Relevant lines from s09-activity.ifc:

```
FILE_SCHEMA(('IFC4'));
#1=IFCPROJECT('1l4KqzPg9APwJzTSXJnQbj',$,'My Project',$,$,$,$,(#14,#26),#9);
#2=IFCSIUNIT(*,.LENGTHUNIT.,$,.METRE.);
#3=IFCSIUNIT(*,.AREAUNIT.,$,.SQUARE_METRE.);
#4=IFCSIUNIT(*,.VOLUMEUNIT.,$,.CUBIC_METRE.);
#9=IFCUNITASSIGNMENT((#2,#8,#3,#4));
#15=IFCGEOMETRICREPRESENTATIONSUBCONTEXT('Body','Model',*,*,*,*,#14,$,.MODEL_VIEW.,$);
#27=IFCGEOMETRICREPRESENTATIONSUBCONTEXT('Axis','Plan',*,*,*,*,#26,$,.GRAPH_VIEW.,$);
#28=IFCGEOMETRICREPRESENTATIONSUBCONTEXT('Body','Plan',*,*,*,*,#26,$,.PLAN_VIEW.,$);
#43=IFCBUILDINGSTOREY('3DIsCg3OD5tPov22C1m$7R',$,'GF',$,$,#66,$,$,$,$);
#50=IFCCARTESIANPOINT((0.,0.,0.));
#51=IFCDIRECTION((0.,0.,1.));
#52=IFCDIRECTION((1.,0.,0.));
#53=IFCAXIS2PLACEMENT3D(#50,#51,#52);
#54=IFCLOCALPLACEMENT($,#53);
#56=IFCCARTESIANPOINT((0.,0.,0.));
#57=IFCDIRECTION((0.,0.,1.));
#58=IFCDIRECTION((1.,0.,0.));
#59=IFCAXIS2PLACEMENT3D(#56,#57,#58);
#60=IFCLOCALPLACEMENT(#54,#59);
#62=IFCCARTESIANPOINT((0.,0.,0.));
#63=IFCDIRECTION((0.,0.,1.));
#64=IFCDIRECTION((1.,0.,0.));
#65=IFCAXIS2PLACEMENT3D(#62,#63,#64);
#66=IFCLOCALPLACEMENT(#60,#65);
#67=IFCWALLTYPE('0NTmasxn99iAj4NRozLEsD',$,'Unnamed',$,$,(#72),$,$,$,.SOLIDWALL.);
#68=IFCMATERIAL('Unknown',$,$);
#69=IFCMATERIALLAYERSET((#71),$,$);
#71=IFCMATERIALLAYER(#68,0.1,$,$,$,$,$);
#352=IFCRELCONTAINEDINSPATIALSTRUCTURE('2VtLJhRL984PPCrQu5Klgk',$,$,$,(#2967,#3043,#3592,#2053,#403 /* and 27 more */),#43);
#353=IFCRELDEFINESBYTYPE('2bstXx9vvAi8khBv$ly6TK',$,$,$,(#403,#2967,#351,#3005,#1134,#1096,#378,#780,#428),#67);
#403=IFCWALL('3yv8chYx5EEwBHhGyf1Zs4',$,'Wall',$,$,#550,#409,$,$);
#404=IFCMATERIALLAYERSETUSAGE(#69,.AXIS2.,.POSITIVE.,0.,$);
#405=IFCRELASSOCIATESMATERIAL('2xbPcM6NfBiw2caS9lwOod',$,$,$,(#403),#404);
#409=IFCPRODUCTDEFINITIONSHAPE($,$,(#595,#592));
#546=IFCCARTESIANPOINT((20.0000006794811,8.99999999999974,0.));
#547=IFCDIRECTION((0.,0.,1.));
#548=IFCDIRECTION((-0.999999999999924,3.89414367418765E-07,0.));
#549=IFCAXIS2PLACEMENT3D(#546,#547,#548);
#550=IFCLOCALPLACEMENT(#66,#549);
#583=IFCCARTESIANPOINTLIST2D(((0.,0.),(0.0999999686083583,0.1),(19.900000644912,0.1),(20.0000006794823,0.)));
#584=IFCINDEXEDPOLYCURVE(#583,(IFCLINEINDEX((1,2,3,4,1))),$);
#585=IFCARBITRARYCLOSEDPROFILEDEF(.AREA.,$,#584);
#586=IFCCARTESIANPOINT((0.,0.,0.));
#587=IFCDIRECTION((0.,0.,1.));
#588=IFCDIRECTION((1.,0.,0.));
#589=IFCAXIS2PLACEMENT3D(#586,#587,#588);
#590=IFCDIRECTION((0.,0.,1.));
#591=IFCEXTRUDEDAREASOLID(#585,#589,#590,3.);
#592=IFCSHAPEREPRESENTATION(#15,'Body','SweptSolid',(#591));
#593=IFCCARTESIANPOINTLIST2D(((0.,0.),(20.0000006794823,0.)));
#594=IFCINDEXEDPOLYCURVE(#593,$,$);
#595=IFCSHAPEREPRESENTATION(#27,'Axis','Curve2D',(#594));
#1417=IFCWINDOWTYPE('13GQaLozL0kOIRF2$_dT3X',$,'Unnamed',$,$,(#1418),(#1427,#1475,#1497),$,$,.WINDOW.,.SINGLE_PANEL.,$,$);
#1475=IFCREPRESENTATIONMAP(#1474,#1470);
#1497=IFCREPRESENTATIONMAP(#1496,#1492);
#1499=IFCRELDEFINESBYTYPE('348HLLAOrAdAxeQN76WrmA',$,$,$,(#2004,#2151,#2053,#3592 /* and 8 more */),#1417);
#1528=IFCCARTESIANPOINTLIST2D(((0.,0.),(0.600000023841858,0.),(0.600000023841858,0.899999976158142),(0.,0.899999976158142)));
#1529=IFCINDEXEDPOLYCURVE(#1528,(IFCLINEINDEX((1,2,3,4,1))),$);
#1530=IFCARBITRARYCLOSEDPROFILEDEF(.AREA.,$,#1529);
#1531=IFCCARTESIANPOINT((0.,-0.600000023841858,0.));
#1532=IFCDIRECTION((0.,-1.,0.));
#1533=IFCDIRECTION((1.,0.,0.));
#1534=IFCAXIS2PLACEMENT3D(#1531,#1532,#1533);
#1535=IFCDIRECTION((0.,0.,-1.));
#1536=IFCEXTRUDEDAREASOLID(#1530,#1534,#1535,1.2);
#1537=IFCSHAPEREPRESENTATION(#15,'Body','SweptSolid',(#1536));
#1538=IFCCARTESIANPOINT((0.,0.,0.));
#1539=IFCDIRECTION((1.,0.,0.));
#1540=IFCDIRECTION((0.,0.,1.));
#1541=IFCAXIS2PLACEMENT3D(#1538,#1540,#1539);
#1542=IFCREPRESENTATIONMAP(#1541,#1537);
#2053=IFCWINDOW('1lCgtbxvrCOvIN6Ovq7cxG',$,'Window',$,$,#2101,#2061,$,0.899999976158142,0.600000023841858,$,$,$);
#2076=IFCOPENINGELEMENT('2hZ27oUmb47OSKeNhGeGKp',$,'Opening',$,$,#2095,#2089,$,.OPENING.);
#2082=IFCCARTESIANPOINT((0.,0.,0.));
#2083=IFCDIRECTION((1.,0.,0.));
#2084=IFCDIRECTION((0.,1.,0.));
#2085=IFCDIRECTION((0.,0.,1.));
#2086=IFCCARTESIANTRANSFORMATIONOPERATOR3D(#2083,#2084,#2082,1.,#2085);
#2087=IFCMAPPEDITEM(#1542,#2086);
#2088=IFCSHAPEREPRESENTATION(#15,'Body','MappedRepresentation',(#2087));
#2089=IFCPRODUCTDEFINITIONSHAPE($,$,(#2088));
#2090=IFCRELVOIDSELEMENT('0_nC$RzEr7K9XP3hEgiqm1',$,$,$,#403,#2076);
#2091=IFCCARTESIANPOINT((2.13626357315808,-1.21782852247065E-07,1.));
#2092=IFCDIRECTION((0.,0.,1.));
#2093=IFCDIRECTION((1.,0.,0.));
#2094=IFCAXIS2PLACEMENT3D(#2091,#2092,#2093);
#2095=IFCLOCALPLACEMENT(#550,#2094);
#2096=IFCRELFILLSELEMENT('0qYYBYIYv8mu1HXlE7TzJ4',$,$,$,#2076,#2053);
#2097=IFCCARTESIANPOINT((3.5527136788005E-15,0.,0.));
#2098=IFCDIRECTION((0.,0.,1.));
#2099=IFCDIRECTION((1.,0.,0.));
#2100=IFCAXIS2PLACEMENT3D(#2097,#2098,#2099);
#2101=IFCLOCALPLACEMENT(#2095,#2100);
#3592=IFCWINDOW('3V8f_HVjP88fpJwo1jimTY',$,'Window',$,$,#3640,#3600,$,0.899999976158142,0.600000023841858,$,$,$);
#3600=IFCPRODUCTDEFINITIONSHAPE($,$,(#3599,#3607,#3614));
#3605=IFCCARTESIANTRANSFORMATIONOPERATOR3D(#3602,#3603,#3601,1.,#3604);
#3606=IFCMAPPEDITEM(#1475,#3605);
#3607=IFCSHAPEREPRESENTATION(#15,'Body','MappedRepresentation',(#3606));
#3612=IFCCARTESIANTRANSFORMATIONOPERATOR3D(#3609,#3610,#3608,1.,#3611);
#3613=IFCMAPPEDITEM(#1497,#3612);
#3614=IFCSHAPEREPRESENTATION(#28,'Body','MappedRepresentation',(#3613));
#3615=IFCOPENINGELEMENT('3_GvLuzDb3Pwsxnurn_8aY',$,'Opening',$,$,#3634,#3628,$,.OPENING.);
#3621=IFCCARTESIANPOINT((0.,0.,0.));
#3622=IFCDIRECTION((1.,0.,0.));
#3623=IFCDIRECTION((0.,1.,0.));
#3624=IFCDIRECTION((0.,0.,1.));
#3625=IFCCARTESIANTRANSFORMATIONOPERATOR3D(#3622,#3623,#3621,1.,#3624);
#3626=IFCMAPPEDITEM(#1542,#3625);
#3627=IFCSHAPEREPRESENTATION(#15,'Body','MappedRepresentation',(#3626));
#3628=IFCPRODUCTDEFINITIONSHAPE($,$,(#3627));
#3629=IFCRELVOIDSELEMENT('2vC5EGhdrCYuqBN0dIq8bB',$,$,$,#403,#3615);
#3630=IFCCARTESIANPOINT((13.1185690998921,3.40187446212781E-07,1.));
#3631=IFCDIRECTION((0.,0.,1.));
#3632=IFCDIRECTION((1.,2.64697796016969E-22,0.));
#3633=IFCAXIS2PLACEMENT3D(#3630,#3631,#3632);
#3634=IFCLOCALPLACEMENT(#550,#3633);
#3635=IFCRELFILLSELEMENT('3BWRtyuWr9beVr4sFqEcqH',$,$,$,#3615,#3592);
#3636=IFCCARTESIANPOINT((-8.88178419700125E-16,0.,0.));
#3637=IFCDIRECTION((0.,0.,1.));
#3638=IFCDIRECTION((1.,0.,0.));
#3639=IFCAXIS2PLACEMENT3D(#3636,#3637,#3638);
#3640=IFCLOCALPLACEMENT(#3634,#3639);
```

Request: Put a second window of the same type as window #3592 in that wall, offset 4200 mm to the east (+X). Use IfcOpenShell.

```python
import ifcopenshell
import ifcopenshell.api.feature
import ifcopenshell.api.geometry
import ifcopenshell.api.root
import ifcopenshell.geom
import ifcopenshell.util.element
import ifcopenshell.util.placement
import ifcopenshell.util.shape

model = ifcopenshell.open("s09-activity.ifc")
settings = ifcopenshell.geom.settings()


def volume(element):
    """Net volume in cubic metres, openings subtracted."""
    shape = ifcopenshell.geom.create_shape(settings, element)
    return ifcopenshell.util.shape.get_volume(shape.geometry)


window = model.by_guid("3V8f_HVjP88fpJwo1jimTY")
opening = window.FillsVoids[0].RelatingOpeningElement
wall = opening.VoidsElements[0].RelatingBuildingElement
before = volume(wall)
shift = ifcopenshell.util.placement.get_local_placement(wall.ObjectPlacement)[:3, 0] * -4.2

# copy_class copies the void relationship, type, container and properties, but no geometry.
new_opening = ifcopenshell.api.root.copy_class(model, product=opening)
new_opening.Representation = ifcopenshell.util.element.copy_deep(
    model, opening.Representation, exclude=["IfcGeometricRepresentationContext", "IfcRepresentationMap"]
)
new_window = ifcopenshell.api.root.copy_class(model, product=window)
new_window.Representation = ifcopenshell.util.element.copy_deep(
    model, window.Representation, exclude=["IfcGeometricRepresentationContext", "IfcRepresentationMap"]
)
ifcopenshell.api.feature.add_filling(model, opening=new_opening, element=new_window)

for old, new in ((opening, new_opening), (window, new_window)):
    matrix = ifcopenshell.util.placement.get_local_placement(old.ObjectPlacement)
    matrix[:3, 3] += shift
    ifcopenshell.api.geometry.edit_object_placement(model, product=new, matrix=matrix, is_si=False)

after = volume(wall)

print(f"wall volume {before:.3f} -> {after:.3f} m3")

model.write("s09-activity_rev.ifc")
```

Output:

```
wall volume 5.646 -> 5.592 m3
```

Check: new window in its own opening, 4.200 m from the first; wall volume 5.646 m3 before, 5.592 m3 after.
